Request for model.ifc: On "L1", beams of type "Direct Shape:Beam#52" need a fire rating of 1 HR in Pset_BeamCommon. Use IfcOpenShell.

First a look at what the model holds.

```python
import ifcopenshell
import ifcopenshell.util.element

model = ifcopenshell.open("model.ifc")
print(model.schema)
storey = next(s for s in model.by_type("IfcBuildingStorey") if s.Name == "L1")
beams = [e for e in ifcopenshell.util.element.get_decomposition(storey) if e.is_a("IfcBeam")]
seen = {}
for e in beams:
    element_type = ifcopenshell.util.element.get_type(e)
    key = (element_type.Name if element_type != e and element_type else None, ifcopenshell.util.element.get_pset(e, "Pset_BeamCommon", "FireRating"))
    seen[key] = seen.get(key, 0) + 1
for (name, value), count in sorted(seen.items(), key=str):
    print(count, "x", name, "|", value)
```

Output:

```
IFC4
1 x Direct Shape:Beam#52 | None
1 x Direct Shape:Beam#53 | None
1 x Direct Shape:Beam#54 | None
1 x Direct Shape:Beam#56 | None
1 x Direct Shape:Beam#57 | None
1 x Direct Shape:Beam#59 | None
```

```python
import ifcopenshell
import ifcopenshell.api.pset
import ifcopenshell.util.element

model = ifcopenshell.open("model.ifc")

storey = next(s for s in model.by_type("IfcBuildingStorey") if s.Name == "L1")
beams = [e for e in ifcopenshell.util.element.get_decomposition(storey) if e.is_a("IfcBeam")]

count = 0
for e in beams:
    element_type = ifcopenshell.util.element.get_type(e)
    if element_type in (None, e) or element_type.Name != "Direct Shape:Beam#52":
        continue
    # add_pset returns the element's existing set when there is one.
    pset = ifcopenshell.api.pset.add_pset(model, product=e, name="Pset_BeamCommon")
    ifcopenshell.api.pset.edit_pset(model, pset=pset, properties={"FireRating": "1 HR"})
    count += 1

print(count, "beams updated")

model.write("model_edited.ifc")
```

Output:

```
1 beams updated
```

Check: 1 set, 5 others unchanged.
